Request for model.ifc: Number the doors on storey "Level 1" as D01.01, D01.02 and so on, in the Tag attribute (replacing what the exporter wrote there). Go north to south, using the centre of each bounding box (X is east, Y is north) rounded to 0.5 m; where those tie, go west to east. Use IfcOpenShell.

First a look at what the model holds.

```python
import ifcopenshell
import ifcopenshell.util.element
import ifcopenshell.util.placement

model = ifcopenshell.open("model.ifc")
print(model.schema)
storey = next(s for s in model.by_type("IfcBuildingStorey") if s.Name == "Level 1")
doors = [e for e in ifcopenshell.util.element.get_decomposition(storey) if e.is_a("IfcDoor")]
for e in sorted(doors, key=lambda e: e.id()):
    origin = ifcopenshell.util.placement.get_local_placement(e.ObjectPlacement)[:3, 3]
    print(e.id(), e.Tag, e.Name, origin.round(2) + 0.0, sep=" | ")
```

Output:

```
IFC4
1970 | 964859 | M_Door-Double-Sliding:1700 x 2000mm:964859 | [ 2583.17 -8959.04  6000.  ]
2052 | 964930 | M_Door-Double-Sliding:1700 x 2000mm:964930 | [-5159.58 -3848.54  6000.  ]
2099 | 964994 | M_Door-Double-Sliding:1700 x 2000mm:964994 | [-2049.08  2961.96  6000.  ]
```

```python
import ifcopenshell
import ifcopenshell.geom
import ifcopenshell.util.element
import ifcopenshell.util.shape

model = ifcopenshell.open("model.ifc")
settings = ifcopenshell.geom.settings()
settings.set("use-world-coords", True)


def centre(element):
    shape = ifcopenshell.geom.create_shape(settings, element)
    return ifcopenshell.util.shape.get_bbox_centroid(shape.geometry)


storey = next(s for s in model.by_type("IfcBuildingStorey") if s.Name == "Level 1")
doors = [e for e in ifcopenshell.util.element.get_decomposition(storey) if e.is_a("IfcDoor")]

# Insertion points can sit at a corner or the storey origin, so sort by the geometry (in metres).
centres = {e: centre(e) for e in doors}
doors.sort(key=lambda e: (-round(centres[e][1] / 0.5), centres[e][0]))

for i, e in enumerate(doors, start=1):
    number = f"D01.{i:02d}"
    e.Tag = number
    print(e.id(), number)

model.write("model_v2.ifc")
```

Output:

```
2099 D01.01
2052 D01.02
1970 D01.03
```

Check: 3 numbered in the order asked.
